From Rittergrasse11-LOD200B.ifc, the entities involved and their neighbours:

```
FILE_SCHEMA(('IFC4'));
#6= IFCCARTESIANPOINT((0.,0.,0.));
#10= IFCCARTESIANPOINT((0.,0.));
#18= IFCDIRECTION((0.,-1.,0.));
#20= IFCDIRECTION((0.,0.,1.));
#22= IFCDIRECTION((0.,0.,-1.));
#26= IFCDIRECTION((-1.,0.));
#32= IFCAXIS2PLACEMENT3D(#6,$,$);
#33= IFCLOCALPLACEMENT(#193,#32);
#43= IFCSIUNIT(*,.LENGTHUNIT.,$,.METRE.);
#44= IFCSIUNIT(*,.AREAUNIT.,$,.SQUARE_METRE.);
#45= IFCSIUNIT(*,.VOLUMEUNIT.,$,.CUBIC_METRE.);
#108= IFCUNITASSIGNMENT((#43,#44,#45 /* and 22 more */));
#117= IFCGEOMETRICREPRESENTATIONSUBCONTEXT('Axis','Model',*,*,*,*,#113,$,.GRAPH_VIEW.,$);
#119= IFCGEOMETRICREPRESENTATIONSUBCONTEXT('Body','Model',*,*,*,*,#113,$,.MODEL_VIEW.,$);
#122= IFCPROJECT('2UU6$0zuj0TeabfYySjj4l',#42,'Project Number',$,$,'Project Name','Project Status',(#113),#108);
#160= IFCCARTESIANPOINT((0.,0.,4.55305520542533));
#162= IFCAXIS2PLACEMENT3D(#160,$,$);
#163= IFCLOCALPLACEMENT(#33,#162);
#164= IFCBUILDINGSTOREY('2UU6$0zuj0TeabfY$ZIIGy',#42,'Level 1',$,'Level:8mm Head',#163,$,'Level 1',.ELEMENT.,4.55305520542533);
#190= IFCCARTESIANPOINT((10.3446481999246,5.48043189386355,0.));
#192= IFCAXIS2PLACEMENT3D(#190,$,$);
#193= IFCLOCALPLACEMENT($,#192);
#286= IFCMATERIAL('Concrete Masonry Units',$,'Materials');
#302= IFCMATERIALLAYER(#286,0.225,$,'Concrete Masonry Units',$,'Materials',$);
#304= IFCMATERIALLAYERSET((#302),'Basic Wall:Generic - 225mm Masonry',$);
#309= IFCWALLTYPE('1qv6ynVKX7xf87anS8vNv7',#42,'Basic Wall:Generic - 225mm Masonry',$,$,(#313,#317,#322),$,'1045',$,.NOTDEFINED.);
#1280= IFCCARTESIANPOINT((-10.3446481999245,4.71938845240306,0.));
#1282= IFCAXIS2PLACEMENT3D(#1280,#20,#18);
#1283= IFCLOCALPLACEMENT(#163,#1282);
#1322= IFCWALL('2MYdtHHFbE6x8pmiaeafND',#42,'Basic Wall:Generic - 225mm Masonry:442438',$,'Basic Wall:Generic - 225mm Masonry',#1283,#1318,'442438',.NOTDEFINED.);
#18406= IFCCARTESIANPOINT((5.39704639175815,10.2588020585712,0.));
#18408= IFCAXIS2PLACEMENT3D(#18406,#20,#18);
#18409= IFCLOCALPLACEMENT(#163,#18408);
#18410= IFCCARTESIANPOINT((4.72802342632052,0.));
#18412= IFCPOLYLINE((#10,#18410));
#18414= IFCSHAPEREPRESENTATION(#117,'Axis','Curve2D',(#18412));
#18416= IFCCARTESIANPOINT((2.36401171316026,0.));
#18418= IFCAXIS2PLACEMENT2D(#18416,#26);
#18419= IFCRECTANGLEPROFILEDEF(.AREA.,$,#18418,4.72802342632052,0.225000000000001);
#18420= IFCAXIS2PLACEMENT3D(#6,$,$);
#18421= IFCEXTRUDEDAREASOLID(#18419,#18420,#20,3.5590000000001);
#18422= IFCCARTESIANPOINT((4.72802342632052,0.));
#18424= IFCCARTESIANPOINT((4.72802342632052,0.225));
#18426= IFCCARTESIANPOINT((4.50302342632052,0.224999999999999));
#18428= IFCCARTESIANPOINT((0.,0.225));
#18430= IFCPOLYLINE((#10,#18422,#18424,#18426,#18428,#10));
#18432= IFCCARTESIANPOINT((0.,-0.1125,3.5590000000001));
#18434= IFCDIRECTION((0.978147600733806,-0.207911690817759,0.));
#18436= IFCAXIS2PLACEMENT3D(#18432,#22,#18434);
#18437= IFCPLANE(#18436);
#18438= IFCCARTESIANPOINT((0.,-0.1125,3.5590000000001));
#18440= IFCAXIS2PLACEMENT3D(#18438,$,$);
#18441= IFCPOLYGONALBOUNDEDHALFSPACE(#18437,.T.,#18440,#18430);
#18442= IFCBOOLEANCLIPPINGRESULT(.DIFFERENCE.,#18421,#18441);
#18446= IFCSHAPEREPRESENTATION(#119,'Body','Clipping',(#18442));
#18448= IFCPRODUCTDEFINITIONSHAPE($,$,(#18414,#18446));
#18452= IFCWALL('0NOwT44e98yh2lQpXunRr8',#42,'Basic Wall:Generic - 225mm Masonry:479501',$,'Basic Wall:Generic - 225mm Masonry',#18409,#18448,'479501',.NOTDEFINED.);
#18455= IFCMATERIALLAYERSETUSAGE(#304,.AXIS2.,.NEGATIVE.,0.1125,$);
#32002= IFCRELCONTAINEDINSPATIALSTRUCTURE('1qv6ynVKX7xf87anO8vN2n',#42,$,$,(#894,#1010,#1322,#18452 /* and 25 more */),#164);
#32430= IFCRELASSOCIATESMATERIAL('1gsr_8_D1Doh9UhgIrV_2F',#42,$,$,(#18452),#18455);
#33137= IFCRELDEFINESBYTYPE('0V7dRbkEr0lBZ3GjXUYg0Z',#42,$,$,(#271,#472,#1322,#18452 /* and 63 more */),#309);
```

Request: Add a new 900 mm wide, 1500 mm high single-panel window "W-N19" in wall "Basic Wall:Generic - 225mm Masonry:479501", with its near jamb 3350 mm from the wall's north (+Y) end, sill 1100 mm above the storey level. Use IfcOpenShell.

```python
import numpy as np
import ifcopenshell
import ifcopenshell.api.feature
import ifcopenshell.api.geometry
import ifcopenshell.api.root
import ifcopenshell.api.spatial
import ifcopenshell.geom
import ifcopenshell.util.element
import ifcopenshell.util.placement
import ifcopenshell.util.representation
import ifcopenshell.util.shape
import ifcopenshell.util.unit

model = ifcopenshell.open("Rittergrasse11-LOD200B.ifc")
unit_scale = ifcopenshell.util.unit.calculate_unit_scale(model)
settings = ifcopenshell.geom.settings()


def volume(element):
    """Net volume in cubic metres, openings subtracted."""
    shape = ifcopenshell.geom.create_shape(settings, element)
    return ifcopenshell.util.shape.get_volume(shape.geometry)


wall = model.by_guid("0NOwT44e98yh2lQpXunRr8")
storey = ifcopenshell.util.element.get_container(wall, ifc_class="IfcBuildingStorey")
context = ifcopenshell.util.representation.get_context(model, "Model", "Body", "MODEL_VIEW")
before = volume(wall)

width, height, from_end, sill = 0.9, 1.5, 3.35, 1.1  # metres

# The wall runs along its own X axis, and the end named is its -X end.
wall_shape = ifcopenshell.geom.create_shape(settings, wall)
x, y, z = ifcopenshell.util.shape.get_vertices(wall_shape.geometry).T
start = x.min() + from_end
face, thickness = float(y.min()), float(y.max() - y.min())
wall_matrix = ifcopenshell.util.placement.get_local_placement(wall.ObjectPlacement)
level = ifcopenshell.util.placement.get_local_placement(storey.ObjectPlacement)[2, 3]


def in_wall(x, y):
    """Placement at x, y metres in the wall's axes, at sill height."""
    matrix = wall_matrix.copy()
    matrix[:, 3] = wall_matrix @ np.array([x / unit_scale, y / unit_scale, 0.0, 1.0])
    matrix[2, 3] = level + sill / unit_scale
    return matrix


# Opening: a box that overshoots both wall faces by 50 mm.
opening = ifcopenshell.api.root.create_entity(model, ifc_class="IfcOpeningElement", predefined_type="OPENING")
box = ifcopenshell.api.geometry.add_wall_representation(
    model, context=context, length=width, height=height, thickness=thickness + 0.1
)
ifcopenshell.api.geometry.assign_representation(model, product=opening, representation=box)
ifcopenshell.api.geometry.edit_object_placement(model, product=opening, matrix=in_wall(start, face - 0.05), is_si=False)
ifcopenshell.api.feature.add_feature(model, feature=opening, element=wall)

window = ifcopenshell.api.root.create_entity(model, ifc_class="IfcWindow", name="W-N19", predefined_type="WINDOW")
window.OverallWidth, window.OverallHeight = width / unit_scale, height / unit_scale
window.PartitioningType = "SINGLE_PANEL"
body = ifcopenshell.api.geometry.add_window_representation(
    model,
    context=context,
    overall_width=window.OverallWidth,
    overall_height=window.OverallHeight,
    partition_type="SINGLE_PANEL",
)
ifcopenshell.api.geometry.assign_representation(model, product=window, representation=body)
ifcopenshell.api.spatial.assign_container(model, products=[window], relating_structure=storey)
ifcopenshell.api.feature.add_filling(model, opening=opening, element=window)

# Centre the window in the wall's thickness.
ifcopenshell.api.geometry.edit_object_placement(model, product=window, matrix=in_wall(start, face), is_si=False)
window_shape = ifcopenshell.geom.create_shape(settings, window)
depth = ifcopenshell.util.shape.get_vertices(window_shape.geometry)[:, 1]
offset = face + thickness / 2 - (depth.min() + depth.max()) / 2
ifcopenshell.api.geometry.edit_object_placement(model, product=window, matrix=in_wall(start, offset), is_si=False)

after = volume(wall)

print(f"wall volume {before:.3f} -> {after:.3f} m3")

model.write("Rittergrasse11-LOD200B-out.ifc")
```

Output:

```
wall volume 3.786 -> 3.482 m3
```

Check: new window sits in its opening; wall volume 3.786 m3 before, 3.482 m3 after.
